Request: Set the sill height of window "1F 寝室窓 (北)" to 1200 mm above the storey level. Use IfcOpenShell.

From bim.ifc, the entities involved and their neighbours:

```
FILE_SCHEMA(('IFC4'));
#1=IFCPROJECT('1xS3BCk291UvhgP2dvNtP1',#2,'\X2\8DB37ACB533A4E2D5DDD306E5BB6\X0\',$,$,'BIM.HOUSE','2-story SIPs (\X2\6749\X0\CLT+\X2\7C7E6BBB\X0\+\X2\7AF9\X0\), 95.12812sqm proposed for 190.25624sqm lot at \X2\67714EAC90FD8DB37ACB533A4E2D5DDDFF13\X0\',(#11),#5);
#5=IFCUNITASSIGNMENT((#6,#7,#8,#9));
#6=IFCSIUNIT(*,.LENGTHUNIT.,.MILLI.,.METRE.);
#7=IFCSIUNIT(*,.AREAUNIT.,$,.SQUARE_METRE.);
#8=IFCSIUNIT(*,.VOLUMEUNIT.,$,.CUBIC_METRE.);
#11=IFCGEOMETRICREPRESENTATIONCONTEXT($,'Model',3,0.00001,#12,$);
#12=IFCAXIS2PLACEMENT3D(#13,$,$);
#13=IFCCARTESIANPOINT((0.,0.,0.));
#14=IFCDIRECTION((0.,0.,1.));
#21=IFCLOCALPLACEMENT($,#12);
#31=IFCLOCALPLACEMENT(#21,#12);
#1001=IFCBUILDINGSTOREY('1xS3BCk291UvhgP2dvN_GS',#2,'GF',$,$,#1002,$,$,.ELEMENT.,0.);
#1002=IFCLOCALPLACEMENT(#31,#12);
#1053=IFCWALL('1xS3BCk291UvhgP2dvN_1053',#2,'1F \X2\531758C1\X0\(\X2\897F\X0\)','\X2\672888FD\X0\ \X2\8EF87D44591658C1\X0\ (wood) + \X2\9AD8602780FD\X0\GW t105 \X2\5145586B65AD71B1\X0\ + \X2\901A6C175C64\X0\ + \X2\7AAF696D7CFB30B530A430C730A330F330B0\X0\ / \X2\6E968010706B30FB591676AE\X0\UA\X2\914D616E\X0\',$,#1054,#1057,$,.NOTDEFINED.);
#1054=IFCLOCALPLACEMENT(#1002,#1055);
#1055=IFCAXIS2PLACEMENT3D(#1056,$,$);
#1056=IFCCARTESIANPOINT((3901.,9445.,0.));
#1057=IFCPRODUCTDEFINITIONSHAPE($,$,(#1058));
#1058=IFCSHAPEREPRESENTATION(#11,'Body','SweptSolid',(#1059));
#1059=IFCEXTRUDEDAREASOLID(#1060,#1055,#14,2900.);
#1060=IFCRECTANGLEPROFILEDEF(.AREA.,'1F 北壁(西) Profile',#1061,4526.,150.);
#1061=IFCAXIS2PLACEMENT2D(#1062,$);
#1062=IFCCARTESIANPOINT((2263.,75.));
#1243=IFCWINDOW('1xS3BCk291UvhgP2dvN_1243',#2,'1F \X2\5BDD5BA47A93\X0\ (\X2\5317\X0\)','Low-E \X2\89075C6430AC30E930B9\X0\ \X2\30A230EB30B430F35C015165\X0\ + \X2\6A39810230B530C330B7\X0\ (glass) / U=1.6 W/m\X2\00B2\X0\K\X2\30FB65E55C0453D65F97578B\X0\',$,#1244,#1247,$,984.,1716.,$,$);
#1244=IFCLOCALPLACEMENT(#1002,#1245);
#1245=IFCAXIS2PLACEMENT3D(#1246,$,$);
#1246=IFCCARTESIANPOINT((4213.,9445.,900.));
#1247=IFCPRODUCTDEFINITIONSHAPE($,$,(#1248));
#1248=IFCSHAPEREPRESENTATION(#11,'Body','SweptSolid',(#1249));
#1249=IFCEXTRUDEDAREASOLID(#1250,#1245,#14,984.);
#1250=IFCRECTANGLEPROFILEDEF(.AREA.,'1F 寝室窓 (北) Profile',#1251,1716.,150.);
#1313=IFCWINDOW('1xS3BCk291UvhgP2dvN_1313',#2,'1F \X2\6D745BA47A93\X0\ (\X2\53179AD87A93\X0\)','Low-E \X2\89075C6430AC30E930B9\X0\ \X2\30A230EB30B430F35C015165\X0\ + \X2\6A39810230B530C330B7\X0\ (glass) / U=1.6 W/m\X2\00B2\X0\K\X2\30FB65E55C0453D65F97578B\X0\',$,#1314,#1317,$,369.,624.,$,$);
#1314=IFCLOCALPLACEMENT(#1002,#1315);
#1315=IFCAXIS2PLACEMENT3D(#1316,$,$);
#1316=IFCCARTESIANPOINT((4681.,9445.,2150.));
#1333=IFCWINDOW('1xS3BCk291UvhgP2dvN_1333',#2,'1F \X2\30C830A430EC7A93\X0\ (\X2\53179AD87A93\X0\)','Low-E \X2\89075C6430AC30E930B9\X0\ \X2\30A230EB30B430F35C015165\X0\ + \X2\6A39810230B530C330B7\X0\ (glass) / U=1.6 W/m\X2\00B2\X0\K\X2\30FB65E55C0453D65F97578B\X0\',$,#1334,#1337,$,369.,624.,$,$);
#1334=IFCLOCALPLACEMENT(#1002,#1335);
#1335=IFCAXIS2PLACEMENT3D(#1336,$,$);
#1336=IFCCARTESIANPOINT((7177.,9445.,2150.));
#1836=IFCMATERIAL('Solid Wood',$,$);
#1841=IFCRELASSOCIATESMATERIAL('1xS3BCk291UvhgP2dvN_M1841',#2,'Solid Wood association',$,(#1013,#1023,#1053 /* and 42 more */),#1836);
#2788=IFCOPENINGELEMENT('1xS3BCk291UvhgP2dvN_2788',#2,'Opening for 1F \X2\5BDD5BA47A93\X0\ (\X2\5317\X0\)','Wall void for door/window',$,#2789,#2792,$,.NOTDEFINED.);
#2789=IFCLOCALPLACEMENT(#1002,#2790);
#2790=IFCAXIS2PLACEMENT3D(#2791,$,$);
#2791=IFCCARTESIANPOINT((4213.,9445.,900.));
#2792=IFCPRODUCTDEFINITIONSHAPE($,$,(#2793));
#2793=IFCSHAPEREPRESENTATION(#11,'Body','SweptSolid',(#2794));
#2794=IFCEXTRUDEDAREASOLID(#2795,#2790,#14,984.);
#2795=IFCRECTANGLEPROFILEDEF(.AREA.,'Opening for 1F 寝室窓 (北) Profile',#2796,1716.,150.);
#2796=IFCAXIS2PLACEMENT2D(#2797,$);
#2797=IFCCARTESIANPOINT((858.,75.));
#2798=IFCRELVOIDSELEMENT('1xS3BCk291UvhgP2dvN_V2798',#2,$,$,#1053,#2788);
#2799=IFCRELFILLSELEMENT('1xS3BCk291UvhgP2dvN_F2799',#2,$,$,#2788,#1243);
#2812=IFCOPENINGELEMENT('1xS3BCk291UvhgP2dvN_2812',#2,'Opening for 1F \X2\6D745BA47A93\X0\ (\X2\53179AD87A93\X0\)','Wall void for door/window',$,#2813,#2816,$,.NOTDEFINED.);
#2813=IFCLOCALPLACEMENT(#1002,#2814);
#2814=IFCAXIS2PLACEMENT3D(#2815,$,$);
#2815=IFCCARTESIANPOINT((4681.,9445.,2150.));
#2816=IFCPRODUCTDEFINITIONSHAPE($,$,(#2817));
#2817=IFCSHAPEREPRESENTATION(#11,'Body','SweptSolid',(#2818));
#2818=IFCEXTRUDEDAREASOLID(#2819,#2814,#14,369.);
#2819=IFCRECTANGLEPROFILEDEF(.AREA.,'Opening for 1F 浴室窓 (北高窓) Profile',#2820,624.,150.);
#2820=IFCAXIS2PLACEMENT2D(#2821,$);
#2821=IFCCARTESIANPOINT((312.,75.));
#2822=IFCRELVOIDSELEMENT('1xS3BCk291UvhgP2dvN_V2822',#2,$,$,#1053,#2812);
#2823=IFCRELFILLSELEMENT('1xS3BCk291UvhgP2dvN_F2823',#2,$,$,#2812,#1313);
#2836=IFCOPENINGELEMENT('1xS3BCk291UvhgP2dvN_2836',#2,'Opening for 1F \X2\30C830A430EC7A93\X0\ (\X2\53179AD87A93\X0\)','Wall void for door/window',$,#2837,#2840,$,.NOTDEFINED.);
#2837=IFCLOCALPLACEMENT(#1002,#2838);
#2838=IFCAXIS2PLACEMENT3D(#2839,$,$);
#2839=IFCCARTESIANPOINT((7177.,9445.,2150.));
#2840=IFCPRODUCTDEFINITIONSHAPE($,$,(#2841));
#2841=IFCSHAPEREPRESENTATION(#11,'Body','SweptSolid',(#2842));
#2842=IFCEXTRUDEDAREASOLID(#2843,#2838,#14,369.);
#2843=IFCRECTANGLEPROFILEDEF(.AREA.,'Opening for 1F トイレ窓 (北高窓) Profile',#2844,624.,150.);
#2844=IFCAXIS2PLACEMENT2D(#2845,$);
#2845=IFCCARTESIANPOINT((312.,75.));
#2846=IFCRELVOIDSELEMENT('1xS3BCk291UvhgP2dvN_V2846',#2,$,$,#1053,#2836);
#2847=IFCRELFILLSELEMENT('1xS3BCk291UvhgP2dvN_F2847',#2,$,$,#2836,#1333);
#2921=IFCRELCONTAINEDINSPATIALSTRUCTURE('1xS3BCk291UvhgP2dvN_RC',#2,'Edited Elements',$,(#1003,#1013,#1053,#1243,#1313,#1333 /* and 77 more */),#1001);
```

```python
import numpy as np
import ifcopenshell
import ifcopenshell.api.geometry
import ifcopenshell.geom
import ifcopenshell.util.element
import ifcopenshell.util.placement
import ifcopenshell.util.shape
import ifcopenshell.util.unit

model = ifcopenshell.open("bim.ifc")
unit_scale = ifcopenshell.util.unit.calculate_unit_scale(model)

window = model.by_guid("1xS3BCk291UvhgP2dvN_1243")
opening = window.FillsVoids[0].RelatingOpeningElement
storey = ifcopenshell.util.element.get_container(window, ifc_class="IfcBuildingStorey")
level = ifcopenshell.util.placement.get_local_placement(storey.ObjectPlacement)[2, 3]

# The opening's origin need not be at the sill, so measure its lowest point.
shape = ifcopenshell.geom.create_shape(ifcopenshell.geom.settings(), opening)
bottom = ifcopenshell.util.shape.get_shape_bottom_elevation(shape, shape.geometry) / unit_scale
dz = level + 1200.0 - bottom

shift = np.array([0.0, 0.0, dz])
# The window is not placed relative to its opening, so move both.
for product in (opening, window):
    matrix = ifcopenshell.util.placement.get_local_placement(product.ObjectPlacement)
    matrix[:3, 3] += shift
    ifcopenshell.api.geometry.edit_object_placement(model, product=product, matrix=matrix, is_si=False)

print(f"moved by {dz * unit_scale:+.3f} m")

model.write("bim-out.ifc")
```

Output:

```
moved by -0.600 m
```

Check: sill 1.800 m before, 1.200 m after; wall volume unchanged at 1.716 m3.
